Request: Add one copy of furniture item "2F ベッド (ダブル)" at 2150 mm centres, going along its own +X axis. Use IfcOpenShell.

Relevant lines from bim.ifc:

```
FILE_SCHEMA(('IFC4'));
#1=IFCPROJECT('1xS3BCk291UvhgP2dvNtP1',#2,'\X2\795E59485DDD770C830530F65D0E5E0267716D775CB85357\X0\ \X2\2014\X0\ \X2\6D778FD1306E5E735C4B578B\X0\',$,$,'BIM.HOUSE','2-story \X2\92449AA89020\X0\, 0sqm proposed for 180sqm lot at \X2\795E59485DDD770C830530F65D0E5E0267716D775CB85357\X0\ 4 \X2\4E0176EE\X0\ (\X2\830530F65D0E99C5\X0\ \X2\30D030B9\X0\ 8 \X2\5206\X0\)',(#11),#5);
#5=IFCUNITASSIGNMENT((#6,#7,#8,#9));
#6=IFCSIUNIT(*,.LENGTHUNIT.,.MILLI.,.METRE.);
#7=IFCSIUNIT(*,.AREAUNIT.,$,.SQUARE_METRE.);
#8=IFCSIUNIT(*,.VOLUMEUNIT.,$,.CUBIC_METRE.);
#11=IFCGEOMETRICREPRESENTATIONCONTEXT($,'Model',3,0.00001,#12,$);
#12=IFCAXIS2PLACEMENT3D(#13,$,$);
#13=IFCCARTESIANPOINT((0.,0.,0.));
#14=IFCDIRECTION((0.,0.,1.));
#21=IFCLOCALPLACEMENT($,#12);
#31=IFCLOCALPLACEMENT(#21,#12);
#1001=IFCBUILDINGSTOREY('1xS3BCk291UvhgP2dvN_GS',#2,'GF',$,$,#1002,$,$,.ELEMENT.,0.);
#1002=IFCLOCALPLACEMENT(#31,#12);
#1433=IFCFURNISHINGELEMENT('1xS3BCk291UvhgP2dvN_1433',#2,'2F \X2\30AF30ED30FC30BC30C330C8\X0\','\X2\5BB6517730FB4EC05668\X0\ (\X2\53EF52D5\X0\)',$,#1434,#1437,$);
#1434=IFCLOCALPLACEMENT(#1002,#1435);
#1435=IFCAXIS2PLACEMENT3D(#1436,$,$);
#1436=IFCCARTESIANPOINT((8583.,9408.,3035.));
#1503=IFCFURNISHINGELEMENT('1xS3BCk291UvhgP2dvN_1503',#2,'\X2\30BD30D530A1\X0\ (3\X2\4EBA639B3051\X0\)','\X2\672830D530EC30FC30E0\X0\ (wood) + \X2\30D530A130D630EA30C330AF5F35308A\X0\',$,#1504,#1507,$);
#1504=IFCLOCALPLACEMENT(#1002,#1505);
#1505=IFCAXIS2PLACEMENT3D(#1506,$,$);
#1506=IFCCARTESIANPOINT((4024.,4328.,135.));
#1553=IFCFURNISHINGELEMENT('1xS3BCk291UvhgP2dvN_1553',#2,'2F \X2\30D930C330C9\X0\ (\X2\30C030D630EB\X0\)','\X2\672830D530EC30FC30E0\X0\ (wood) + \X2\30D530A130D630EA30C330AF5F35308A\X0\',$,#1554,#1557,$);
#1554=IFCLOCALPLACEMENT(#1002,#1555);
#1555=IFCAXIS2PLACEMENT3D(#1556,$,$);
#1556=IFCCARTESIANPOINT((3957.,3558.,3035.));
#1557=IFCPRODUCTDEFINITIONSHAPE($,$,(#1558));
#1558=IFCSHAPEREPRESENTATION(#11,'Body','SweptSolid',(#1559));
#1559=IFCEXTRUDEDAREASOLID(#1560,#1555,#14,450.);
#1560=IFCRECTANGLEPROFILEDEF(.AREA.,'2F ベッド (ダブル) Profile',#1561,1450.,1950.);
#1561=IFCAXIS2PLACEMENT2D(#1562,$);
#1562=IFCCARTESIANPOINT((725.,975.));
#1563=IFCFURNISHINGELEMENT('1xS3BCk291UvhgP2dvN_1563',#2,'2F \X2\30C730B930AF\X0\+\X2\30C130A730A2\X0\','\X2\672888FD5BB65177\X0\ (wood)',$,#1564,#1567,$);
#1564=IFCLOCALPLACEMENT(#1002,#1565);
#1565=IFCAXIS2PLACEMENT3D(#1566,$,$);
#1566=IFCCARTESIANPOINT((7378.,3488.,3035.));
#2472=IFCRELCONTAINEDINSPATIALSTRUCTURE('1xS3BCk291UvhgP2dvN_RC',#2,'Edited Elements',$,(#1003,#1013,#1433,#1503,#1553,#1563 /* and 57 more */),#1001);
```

```python
import ifcopenshell
import ifcopenshell.api.geometry
import ifcopenshell.api.root
import ifcopenshell.util.element
import ifcopenshell.util.placement

model = ifcopenshell.open("bim.ifc")


def reuse_history(source, copy):
    """copy_class also copies each property set's owner history, people and application; keep the originals."""
    for rel in copy.IsDefinedBy:
        if rel.is_a("IfcRelDefinesByProperties") and (history := rel.RelatingPropertyDefinition.OwnerHistory):
            rel.RelatingPropertyDefinition.OwnerHistory = source.OwnerHistory
            ifcopenshell.util.element.remove_deep2(model, history)


source = model.by_id(1553)
base = ifcopenshell.util.placement.get_local_placement(source.ObjectPlacement)
step = base[:3, 0] * 2150.0

for i in range(1, 2):
    copy = ifcopenshell.api.root.copy_class(model, product=source)
    copy.Representation = ifcopenshell.util.element.copy_deep(
        model, source.Representation, exclude=["IfcGeometricRepresentationContext", "IfcRepresentationMap"]
    )
    reuse_history(source, copy)
    matrix = base.copy()
    matrix[:3, 3] += i * step
    print("added at", matrix[:3, 3].round(3) + 0.0)
    ifcopenshell.api.geometry.edit_object_placement(model, product=copy, matrix=matrix, is_si=False)

model.write("bim_edited.ifc")
```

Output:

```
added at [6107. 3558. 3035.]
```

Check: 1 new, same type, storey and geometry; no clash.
